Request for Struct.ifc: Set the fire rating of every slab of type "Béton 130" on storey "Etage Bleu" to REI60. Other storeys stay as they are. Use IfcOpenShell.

First a look at what the model holds.

```python
import ifcopenshell
import ifcopenshell.util.element

model = ifcopenshell.open("Struct.ifc")
print(model.schema)
storey = next(s for s in model.by_type("IfcBuildingStorey") if s.Name == "Etage Bleu")
slabs = [e for e in ifcopenshell.util.element.get_decomposition(storey) if e.is_a("IfcSlab")]
seen = {}
for e in slabs:
    element_type = ifcopenshell.util.element.get_type(e)
    key = (element_type.Name if element_type != e and element_type else None, ifcopenshell.util.element.get_pset(e, "Pset_SlabCommon", "FireRating"))
    seen[key] = seen.get(key, 0) + 1
for (name, value), count in sorted(seen.items(), key=str):
    print(count, "x", name, "|", value)
```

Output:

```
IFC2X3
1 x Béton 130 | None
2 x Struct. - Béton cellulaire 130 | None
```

```python
import ifcopenshell
import ifcopenshell.api.pset
import ifcopenshell.util.element

model = ifcopenshell.open("Struct.ifc")

storey = next(s for s in model.by_type("IfcBuildingStorey") if s.Name == "Etage Bleu")
slabs = [e for e in ifcopenshell.util.element.get_decomposition(storey) if e.is_a("IfcSlab")]

count = 0
for e in slabs:
    element_type = ifcopenshell.util.element.get_type(e)
    if element_type in (None, e) or element_type.Name != "Béton 130":
        continue
    # add_pset returns the element's existing set when there is one.
    pset = ifcopenshell.api.pset.add_pset(model, product=e, name="Pset_SlabCommon")
    ifcopenshell.api.pset.edit_pset(model, pset=pset, properties={"FireRating": "REI60"})
    count += 1

print(count, "slabs updated")

model.write("Struct-out.ifc")
```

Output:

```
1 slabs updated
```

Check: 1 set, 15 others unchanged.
